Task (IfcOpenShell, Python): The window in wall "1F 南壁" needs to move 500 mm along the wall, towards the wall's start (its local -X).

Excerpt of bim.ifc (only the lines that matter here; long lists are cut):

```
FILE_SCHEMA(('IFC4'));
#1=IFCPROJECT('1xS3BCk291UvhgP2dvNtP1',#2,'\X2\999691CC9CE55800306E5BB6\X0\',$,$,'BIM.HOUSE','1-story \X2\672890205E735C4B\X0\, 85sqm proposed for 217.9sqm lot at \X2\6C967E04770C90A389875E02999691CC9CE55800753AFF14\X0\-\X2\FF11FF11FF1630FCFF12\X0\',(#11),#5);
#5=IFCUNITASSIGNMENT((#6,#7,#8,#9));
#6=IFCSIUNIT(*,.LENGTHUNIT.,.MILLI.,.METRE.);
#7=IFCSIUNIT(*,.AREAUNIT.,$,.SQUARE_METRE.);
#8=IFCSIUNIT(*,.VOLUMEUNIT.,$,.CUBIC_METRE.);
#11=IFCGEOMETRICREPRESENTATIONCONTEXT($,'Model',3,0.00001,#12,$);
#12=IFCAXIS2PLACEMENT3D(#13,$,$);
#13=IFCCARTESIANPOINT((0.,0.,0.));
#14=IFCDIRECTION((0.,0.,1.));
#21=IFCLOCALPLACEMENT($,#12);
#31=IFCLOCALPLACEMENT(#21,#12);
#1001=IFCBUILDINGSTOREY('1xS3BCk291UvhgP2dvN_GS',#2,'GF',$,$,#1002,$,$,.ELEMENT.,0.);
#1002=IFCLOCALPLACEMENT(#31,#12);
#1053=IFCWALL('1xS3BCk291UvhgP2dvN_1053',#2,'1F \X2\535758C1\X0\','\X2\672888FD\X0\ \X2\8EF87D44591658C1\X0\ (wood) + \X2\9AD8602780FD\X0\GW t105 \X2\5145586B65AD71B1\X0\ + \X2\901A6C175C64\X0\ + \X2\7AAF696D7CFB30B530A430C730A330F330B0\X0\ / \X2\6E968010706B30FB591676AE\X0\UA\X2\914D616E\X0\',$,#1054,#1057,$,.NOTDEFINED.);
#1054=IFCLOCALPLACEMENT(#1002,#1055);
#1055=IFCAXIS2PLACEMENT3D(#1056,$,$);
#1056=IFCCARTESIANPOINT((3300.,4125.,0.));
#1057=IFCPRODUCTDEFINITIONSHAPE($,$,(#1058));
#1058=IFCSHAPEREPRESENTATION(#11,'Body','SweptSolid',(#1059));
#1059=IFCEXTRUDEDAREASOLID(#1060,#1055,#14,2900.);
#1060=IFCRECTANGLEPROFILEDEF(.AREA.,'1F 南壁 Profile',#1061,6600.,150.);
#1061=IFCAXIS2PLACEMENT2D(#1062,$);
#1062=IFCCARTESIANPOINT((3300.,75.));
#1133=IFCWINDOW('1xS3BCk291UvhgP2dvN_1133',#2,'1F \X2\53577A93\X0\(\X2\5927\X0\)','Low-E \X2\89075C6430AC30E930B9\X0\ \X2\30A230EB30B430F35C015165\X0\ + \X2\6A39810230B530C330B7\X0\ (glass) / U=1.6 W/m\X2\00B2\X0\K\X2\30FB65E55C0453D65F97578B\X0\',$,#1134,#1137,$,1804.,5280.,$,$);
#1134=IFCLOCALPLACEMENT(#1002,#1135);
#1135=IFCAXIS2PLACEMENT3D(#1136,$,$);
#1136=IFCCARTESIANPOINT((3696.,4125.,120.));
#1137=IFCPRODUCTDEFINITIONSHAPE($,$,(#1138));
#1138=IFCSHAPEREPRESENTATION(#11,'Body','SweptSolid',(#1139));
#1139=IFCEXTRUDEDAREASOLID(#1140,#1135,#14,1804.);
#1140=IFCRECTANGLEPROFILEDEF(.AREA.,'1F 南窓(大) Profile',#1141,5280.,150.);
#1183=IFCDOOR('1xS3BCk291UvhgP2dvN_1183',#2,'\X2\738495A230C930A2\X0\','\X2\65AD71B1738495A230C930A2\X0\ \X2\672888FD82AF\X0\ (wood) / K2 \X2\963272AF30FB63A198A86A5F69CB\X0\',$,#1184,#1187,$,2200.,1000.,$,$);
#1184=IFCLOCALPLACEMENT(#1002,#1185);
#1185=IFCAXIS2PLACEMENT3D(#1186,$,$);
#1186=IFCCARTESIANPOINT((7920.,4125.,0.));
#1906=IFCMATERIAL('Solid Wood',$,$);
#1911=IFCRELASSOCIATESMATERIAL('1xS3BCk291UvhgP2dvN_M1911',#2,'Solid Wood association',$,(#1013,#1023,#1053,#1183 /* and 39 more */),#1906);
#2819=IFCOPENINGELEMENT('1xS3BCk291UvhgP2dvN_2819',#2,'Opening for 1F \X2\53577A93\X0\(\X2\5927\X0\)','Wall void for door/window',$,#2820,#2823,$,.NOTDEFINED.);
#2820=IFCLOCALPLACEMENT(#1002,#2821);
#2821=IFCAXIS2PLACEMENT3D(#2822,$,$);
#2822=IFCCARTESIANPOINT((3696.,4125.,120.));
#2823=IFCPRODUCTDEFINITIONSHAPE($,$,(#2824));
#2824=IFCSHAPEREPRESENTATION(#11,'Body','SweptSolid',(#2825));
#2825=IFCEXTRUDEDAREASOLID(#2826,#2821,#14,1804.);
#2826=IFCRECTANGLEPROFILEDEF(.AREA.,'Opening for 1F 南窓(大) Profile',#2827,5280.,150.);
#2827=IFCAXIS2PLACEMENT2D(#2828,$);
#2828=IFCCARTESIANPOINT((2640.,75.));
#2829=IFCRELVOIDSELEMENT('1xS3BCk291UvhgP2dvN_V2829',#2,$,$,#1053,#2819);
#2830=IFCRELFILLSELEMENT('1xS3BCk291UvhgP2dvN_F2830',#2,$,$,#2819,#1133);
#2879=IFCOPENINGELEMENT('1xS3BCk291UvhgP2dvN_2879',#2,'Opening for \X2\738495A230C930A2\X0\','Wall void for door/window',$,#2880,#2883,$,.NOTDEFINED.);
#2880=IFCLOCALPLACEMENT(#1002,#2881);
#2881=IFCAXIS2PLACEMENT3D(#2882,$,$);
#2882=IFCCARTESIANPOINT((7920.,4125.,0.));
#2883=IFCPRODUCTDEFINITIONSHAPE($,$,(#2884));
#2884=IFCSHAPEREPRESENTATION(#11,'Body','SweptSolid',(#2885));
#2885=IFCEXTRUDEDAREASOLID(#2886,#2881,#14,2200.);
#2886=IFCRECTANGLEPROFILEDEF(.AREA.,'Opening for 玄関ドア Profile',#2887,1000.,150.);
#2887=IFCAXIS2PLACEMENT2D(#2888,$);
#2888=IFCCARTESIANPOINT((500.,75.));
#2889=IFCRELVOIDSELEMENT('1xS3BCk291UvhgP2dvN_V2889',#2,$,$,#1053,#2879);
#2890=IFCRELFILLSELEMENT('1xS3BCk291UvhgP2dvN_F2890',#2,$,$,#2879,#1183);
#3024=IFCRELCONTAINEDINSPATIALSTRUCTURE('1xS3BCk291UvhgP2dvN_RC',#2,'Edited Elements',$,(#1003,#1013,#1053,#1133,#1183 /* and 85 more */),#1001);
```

```python
import ifcopenshell
import ifcopenshell.api.geometry
import ifcopenshell.util.placement

model = ifcopenshell.open("bim.ifc")

window = model.by_guid("1xS3BCk291UvhgP2dvN_1133")
opening = window.FillsVoids[0].RelatingOpeningElement
wall = opening.VoidsElements[0].RelatingBuildingElement

wall_matrix = ifcopenshell.util.placement.get_local_placement(wall.ObjectPlacement)
shift = wall_matrix[:3, 0] * -500.0
before = ifcopenshell.util.placement.get_local_placement(window.ObjectPlacement)[:3, 3].copy()

# The window is not placed relative to its opening, so move both.
for product in (opening, window):
    matrix = ifcopenshell.util.placement.get_local_placement(product.ObjectPlacement)
    matrix[:3, 3] += shift
    ifcopenshell.api.geometry.edit_object_placement(model, product=product, matrix=matrix, is_si=False)

after = ifcopenshell.util.placement.get_local_placement(window.ObjectPlacement)[:3, 3]
print("window moved by", (after - before).round(3) + 0.0)

model.write("bim_v2.ifc")
```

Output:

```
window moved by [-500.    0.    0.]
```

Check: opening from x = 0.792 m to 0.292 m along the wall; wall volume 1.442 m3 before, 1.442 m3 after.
